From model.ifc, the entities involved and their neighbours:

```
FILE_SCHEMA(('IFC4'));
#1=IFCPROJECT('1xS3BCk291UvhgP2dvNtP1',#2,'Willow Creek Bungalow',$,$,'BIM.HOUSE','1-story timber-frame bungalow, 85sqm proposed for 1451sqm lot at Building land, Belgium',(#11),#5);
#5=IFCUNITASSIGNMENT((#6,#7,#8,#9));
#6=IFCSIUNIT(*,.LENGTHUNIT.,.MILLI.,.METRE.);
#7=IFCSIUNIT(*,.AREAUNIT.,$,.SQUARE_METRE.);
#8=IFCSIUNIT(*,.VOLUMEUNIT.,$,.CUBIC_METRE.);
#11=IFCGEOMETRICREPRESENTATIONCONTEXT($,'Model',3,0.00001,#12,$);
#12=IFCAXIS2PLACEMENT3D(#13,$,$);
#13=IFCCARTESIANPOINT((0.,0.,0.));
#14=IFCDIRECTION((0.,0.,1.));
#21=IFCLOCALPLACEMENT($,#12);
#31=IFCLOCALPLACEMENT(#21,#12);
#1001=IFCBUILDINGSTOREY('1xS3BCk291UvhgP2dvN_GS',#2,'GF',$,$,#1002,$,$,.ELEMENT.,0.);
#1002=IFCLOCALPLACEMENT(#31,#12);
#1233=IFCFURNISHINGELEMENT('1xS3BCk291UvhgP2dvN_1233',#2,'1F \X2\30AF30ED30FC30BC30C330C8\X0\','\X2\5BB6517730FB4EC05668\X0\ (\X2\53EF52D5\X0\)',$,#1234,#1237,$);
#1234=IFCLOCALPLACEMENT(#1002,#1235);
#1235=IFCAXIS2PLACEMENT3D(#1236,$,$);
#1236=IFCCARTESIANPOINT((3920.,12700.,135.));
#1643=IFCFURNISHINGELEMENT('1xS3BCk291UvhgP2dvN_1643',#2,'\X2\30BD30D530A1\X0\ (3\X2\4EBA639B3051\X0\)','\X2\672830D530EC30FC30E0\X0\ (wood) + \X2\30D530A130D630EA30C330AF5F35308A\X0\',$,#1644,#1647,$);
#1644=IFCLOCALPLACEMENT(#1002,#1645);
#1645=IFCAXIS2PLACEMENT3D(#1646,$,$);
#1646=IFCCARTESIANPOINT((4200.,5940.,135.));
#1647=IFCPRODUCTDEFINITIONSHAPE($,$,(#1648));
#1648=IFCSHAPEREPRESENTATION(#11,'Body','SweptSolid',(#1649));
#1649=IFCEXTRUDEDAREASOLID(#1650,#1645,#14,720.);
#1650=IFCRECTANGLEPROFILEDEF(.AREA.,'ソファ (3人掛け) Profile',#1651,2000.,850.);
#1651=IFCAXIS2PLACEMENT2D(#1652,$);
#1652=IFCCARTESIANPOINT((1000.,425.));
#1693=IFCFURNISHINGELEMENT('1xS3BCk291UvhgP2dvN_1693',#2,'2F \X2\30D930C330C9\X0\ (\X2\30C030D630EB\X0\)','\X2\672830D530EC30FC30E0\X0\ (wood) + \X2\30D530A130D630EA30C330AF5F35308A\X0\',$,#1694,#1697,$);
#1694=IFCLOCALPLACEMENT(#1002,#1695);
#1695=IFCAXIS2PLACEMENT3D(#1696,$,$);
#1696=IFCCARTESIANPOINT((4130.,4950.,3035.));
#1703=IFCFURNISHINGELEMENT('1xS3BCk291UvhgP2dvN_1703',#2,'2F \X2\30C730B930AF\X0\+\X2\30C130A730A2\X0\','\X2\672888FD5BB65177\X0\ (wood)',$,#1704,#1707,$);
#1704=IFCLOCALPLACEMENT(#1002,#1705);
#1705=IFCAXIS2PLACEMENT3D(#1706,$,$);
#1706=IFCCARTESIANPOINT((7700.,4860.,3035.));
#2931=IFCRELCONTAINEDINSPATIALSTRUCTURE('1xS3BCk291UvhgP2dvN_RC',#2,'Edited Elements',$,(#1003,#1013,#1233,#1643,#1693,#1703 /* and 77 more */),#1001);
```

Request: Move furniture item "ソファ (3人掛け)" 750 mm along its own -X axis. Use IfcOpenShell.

```python
import ifcopenshell
import ifcopenshell.api.geometry
import ifcopenshell.util.placement
import ifcopenshell.util.unit

model = ifcopenshell.open("model.ifc")
unit_scale = ifcopenshell.util.unit.calculate_unit_scale(model)

item = model.by_guid("1xS3BCk291UvhgP2dvN_1643")
matrix = ifcopenshell.util.placement.get_local_placement(item.ObjectPlacement)
matrix[:3, 3] -= matrix[:3, 0] * 0.75 / unit_scale
ifcopenshell.api.geometry.edit_object_placement(model, product=item, matrix=matrix, is_si=False)

print(ifcopenshell.util.placement.get_local_placement(item.ObjectPlacement).round(3) + 0.0)

model.write("model_rev.ifc")
```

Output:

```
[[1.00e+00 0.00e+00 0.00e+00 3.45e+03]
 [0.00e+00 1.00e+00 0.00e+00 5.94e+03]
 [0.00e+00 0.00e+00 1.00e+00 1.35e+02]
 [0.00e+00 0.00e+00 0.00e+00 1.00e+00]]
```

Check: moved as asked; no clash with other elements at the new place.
